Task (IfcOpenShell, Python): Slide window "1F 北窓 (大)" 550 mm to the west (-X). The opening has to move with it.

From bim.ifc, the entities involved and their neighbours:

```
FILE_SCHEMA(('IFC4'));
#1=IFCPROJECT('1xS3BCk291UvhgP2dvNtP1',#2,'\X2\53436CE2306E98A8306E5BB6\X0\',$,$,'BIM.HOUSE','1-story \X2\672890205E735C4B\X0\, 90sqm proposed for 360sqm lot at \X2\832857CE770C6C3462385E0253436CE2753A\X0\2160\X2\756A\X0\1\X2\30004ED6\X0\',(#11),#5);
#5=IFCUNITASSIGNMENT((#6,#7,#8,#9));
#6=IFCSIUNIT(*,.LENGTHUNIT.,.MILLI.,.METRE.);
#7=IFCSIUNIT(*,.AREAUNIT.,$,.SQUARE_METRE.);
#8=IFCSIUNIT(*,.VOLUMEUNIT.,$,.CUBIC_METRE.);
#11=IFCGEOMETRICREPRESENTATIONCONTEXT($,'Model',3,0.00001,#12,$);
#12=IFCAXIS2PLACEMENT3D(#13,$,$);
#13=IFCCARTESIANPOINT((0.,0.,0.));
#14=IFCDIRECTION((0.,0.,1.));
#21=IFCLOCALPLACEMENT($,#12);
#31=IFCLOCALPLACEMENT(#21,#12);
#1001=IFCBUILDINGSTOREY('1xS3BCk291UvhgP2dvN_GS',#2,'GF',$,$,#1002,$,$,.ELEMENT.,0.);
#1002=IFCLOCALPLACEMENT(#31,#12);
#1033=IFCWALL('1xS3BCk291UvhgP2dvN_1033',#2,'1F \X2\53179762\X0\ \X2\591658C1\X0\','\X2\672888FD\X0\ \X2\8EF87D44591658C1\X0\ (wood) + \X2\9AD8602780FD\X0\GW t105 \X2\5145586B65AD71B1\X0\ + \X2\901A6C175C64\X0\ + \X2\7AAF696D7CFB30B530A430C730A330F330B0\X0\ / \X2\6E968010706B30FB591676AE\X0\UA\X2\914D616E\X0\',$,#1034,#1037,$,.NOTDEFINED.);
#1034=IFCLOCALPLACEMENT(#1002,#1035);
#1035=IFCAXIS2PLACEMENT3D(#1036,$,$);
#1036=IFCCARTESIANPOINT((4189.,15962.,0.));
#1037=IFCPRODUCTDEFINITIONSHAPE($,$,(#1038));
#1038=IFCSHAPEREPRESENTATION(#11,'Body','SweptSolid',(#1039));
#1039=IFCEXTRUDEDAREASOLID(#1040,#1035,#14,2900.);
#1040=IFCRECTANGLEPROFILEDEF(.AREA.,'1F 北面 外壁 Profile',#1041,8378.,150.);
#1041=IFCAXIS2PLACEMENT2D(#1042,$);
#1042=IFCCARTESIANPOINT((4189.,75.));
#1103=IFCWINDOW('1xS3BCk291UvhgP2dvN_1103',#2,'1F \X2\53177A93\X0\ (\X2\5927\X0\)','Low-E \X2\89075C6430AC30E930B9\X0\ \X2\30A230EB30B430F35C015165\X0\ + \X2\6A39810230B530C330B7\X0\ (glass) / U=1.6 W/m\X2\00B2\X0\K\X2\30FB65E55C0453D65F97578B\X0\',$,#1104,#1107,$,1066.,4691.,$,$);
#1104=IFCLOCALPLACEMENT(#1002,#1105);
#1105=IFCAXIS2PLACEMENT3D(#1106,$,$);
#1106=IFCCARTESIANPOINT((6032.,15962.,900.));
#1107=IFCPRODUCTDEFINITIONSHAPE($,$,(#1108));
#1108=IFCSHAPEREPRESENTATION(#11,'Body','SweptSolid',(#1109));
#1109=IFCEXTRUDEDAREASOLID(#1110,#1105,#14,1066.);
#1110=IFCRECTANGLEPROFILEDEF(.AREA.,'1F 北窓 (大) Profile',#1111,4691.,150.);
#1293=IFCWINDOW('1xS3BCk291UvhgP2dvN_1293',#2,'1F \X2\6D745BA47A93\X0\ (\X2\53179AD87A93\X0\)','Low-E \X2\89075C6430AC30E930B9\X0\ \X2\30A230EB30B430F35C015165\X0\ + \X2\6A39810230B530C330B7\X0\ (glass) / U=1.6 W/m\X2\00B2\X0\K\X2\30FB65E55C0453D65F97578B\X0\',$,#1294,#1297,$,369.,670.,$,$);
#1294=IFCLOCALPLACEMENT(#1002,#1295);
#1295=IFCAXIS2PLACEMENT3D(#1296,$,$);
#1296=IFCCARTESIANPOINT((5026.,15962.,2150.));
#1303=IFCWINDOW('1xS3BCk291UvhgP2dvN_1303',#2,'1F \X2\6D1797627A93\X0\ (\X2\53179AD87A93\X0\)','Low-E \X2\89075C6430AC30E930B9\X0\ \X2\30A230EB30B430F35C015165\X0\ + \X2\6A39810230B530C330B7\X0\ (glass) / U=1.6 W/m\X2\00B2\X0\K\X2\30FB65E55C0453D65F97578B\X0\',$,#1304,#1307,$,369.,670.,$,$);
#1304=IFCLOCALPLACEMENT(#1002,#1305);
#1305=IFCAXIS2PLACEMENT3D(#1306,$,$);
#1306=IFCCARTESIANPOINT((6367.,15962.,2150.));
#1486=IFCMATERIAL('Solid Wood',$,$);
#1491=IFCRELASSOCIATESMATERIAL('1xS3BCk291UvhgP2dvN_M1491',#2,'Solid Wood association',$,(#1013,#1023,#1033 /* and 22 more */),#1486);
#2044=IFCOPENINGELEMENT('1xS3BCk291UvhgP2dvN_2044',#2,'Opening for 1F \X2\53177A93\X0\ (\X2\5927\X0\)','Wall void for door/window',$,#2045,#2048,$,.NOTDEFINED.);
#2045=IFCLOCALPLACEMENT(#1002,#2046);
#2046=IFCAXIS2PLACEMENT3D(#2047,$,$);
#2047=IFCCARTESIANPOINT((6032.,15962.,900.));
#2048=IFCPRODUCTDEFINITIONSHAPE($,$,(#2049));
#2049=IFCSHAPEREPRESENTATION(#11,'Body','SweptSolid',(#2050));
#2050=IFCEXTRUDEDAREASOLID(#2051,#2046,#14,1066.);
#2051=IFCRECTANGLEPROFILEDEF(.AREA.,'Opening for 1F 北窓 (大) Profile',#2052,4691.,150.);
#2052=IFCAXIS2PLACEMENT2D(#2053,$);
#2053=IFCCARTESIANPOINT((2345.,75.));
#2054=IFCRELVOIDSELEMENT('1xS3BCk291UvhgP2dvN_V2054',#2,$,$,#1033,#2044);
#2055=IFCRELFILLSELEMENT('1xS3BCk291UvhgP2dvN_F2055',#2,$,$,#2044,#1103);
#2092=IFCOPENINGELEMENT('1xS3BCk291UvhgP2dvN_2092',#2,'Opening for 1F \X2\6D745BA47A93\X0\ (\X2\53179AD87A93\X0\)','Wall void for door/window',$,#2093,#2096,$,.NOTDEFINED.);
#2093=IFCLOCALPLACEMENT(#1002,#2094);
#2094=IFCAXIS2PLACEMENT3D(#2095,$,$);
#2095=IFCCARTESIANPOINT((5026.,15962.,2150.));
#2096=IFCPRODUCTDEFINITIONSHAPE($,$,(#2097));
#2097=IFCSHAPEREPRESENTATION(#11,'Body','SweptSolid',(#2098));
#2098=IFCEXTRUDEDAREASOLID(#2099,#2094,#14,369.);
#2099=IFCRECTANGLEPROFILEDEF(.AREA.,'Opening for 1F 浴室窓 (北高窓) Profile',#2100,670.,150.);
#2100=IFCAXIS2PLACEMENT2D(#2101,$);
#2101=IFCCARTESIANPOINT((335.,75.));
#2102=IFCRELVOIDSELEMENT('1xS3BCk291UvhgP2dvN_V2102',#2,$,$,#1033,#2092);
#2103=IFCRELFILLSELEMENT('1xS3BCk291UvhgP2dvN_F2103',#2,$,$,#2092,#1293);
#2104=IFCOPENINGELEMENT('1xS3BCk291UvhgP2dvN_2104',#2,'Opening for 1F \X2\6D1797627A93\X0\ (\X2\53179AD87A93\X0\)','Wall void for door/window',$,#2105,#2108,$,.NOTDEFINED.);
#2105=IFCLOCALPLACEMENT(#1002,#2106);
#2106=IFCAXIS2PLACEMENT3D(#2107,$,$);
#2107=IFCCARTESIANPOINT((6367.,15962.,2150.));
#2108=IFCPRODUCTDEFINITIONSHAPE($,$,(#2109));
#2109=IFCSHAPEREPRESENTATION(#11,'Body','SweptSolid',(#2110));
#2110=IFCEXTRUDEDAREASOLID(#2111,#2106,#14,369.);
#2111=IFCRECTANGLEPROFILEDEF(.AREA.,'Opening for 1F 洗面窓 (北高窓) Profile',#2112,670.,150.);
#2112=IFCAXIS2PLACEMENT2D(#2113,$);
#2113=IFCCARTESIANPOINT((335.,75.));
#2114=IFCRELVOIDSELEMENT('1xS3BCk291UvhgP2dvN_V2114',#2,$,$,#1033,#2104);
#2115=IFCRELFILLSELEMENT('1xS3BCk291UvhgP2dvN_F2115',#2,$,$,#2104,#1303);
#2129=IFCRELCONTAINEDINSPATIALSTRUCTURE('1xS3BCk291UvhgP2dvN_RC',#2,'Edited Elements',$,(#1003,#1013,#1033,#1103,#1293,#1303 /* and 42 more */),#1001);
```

```python
import ifcopenshell
import ifcopenshell.api.geometry
import ifcopenshell.util.placement
import ifcopenshell.util.unit

model = ifcopenshell.open("bim.ifc")
unit_scale = ifcopenshell.util.unit.calculate_unit_scale(model)

window = model.by_guid("1xS3BCk291UvhgP2dvN_1103")
opening = window.FillsVoids[0].RelatingOpeningElement
wall = opening.VoidsElements[0].RelatingBuildingElement

wall_matrix = ifcopenshell.util.placement.get_local_placement(wall.ObjectPlacement)
shift = wall_matrix[:3, 0] * -0.55 / unit_scale
before = ifcopenshell.util.placement.get_local_placement(window.ObjectPlacement)[:3, 3].copy()

# The window is not placed relative to its opening, so move both.
for product in (opening, window):
    matrix = ifcopenshell.util.placement.get_local_placement(product.ObjectPlacement)
    matrix[:3, 3] += shift
    ifcopenshell.api.geometry.edit_object_placement(model, product=product, matrix=matrix, is_si=False)

after = ifcopenshell.util.placement.get_local_placement(window.ObjectPlacement)[:3, 3]
print("window moved by", (after - before).round(3) + 0.0)

model.write("bim-out.ifc")
```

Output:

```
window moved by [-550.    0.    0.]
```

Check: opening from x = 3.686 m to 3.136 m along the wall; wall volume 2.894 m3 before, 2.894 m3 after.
